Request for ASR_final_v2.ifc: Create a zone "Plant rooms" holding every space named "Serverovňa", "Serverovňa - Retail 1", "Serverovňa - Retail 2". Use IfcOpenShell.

First a look at what the model holds.

```python
import ifcopenshell

model = ifcopenshell.open("ASR_final_v2.ifc")
print(model.schema)
seen = {}
for space in model.by_type("IfcSpace"):
    seen[space.LongName] = seen.get(space.LongName, 0) + 1
for name, count in sorted(seen.items(), key=str):
    print(count, "x", name)
print("zones:", [z.Name for z in model.by_type("IfcZone")][:20])
```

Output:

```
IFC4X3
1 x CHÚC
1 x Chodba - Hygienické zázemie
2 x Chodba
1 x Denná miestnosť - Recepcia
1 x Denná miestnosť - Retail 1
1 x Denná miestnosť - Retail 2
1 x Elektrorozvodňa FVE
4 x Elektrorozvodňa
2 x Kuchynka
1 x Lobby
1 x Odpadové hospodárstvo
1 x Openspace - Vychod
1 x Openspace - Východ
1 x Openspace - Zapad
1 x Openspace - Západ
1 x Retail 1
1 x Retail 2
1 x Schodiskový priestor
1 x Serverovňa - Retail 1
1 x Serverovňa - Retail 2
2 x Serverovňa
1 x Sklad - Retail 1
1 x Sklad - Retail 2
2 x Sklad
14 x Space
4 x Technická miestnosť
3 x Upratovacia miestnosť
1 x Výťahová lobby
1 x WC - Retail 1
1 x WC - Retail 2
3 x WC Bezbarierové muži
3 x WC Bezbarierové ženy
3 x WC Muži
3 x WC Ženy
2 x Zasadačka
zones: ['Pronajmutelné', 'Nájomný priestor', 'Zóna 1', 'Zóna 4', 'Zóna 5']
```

```python
import ifcopenshell
import ifcopenshell.api.group
import ifcopenshell.api.root

model = ifcopenshell.open("ASR_final_v2.ifc")

names = {"Serverovňa", "Serverovňa - Retail 1", "Serverovňa - Retail 2"}
spaces = [s for s in model.by_type("IfcSpace") if s.LongName in names]

zone = ifcopenshell.api.root.create_entity(model, ifc_class="IfcZone", name="Plant rooms")
ifcopenshell.api.group.assign_group(model, products=spaces, group=zone)
print(len(spaces), "spaces in", zone.Name)

model.write("ASR_final_v2_rev.ifc")
```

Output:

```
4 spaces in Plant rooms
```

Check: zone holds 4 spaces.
